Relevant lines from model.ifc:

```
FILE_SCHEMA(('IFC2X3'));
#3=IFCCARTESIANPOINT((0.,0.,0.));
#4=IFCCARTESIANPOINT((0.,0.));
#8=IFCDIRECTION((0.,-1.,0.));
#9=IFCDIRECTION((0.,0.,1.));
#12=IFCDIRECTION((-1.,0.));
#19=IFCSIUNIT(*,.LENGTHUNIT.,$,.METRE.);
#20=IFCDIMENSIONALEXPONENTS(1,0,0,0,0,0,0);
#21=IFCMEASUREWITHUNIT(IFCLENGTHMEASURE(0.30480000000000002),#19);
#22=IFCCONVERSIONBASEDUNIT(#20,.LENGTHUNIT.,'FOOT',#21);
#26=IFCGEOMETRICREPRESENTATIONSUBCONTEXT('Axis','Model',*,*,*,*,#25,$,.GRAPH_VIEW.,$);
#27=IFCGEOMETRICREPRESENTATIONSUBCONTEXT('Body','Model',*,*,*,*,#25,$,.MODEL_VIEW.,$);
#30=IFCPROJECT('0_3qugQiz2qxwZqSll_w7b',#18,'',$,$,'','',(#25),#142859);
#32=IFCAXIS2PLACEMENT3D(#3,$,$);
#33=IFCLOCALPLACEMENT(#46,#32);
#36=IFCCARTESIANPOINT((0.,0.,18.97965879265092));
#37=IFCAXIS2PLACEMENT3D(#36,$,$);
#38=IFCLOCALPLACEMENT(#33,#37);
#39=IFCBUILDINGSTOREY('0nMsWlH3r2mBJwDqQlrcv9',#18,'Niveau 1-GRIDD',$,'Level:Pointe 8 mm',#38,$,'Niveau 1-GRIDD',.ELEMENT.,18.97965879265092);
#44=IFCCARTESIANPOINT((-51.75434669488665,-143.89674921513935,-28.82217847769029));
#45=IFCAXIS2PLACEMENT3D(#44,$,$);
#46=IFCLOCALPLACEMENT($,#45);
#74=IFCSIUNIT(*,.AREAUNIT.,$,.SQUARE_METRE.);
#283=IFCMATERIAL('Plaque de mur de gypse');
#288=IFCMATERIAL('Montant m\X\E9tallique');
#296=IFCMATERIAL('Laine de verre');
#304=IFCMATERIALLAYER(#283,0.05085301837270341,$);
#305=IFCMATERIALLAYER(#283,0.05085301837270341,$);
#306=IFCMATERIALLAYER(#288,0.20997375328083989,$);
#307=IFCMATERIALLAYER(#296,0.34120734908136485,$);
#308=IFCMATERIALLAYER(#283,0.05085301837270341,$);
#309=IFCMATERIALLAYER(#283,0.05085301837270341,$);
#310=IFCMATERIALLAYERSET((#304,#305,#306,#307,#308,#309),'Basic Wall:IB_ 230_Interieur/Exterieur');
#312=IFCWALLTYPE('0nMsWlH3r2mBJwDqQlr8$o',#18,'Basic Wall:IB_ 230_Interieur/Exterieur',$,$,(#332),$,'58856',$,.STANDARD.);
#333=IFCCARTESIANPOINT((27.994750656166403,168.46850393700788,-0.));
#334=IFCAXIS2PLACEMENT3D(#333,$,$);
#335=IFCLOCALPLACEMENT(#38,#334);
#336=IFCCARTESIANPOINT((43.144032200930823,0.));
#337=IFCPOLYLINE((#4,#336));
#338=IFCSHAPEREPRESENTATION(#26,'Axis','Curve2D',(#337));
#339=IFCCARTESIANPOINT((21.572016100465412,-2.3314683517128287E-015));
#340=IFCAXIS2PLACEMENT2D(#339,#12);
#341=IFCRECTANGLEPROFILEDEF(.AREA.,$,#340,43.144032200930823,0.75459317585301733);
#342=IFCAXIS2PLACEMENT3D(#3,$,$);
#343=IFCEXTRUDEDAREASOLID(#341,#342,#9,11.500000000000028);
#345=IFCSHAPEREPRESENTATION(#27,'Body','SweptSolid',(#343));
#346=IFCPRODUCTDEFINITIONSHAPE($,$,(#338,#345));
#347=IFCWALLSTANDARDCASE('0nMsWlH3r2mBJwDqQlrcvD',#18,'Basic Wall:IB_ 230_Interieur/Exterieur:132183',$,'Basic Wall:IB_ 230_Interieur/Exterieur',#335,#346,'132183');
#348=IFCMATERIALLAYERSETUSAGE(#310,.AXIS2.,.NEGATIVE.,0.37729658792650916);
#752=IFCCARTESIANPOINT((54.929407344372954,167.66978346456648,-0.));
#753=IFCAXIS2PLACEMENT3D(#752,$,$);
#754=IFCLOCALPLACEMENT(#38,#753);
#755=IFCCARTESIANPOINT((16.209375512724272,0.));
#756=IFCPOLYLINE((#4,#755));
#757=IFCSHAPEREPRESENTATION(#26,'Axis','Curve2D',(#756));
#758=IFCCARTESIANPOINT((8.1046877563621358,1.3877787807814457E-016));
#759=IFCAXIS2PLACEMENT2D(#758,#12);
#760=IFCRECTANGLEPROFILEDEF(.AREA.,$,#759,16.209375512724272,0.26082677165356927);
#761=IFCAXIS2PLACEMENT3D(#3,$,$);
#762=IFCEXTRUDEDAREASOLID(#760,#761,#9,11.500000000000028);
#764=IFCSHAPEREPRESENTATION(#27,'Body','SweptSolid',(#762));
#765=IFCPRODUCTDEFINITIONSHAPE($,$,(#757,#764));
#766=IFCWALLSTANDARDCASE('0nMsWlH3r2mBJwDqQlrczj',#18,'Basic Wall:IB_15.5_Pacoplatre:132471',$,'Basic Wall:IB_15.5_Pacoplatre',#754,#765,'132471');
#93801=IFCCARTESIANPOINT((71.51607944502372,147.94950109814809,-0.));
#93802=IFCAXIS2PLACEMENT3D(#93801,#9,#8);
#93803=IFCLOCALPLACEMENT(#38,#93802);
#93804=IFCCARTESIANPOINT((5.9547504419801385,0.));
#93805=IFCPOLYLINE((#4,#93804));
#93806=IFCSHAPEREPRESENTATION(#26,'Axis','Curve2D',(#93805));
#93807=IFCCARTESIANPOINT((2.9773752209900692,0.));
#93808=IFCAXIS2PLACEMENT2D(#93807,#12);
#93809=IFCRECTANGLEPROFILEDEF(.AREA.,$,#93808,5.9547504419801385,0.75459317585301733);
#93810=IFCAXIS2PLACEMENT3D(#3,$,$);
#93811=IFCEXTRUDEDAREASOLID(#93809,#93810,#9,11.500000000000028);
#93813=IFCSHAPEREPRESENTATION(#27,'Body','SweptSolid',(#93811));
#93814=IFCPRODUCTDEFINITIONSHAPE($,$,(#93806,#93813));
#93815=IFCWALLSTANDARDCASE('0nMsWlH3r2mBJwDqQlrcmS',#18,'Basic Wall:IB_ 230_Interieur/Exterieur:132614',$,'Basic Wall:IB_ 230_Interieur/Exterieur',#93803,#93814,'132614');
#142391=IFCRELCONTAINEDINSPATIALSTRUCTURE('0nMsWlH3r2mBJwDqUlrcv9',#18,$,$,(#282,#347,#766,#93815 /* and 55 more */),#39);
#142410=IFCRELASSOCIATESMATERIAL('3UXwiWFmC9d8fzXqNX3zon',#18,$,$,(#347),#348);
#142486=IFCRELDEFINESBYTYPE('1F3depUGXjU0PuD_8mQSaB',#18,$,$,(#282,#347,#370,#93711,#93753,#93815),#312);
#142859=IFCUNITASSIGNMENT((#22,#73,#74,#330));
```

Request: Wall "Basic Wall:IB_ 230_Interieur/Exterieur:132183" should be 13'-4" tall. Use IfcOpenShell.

```python
import ifcopenshell
import ifcopenshell.geom
import ifcopenshell.util.representation
import ifcopenshell.util.shape
import ifcopenshell.util.unit

model = ifcopenshell.open("model.ifc")
unit_scale = ifcopenshell.util.unit.calculate_unit_scale(model)
settings = ifcopenshell.geom.settings()


def volume(element):
    """Net volume in cubic metres, openings subtracted."""
    shape = ifcopenshell.geom.create_shape(settings, element)
    return ifcopenshell.util.shape.get_volume(shape.geometry)


wall = model.by_guid("0nMsWlH3r2mBJwDqQlrcvD")
before = volume(wall)

body = ifcopenshell.util.representation.get_representation(wall, "Model", "Body")
solid = body.Items[0]
old_height = solid.Depth
solid.Depth = 160 * 0.0254 / unit_scale
after = volume(wall)

print(f"height {old_height:g} -> {solid.Depth:g}, volume {before:.3f} -> {after:.3f} m3")

model.write("model-out.ifc")
```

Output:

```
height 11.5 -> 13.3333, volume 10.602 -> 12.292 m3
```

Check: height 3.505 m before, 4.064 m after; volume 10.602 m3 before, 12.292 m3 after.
